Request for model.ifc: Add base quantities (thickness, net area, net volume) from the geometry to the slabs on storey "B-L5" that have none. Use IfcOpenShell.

First a look at what the model holds.

```python
import ifcopenshell
import ifcopenshell.util.element
import ifcopenshell.util.unit

model = ifcopenshell.open("model.ifc")
print(model.schema)
for unit_type in ("LENGTHUNIT", "AREAUNIT", "VOLUMEUNIT"):
    print(unit_type, ifcopenshell.util.unit.calculate_unit_scale(model, unit_type))
storey = next(s for s in model.by_type("IfcBuildingStorey") if s.Name == "B-L5")
slabs = [e for e in ifcopenshell.util.element.get_decomposition(storey) if e.is_a("IfcSlab")]
for e in sorted(slabs, key=lambda e: e.id()):
    print(e.id(), e.is_a(), e.Name, list(ifcopenshell.util.element.get_psets(e, qtos_only=True)), sep=" | ")
```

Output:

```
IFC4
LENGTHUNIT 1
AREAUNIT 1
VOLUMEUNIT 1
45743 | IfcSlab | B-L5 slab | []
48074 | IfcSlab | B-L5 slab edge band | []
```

```python
import ifcopenshell
import ifcopenshell.api.pset
import ifcopenshell.geom
import ifcopenshell.util.element
import ifcopenshell.util.shape
import ifcopenshell.util.unit

model = ifcopenshell.open("model.ifc")
unit_scale = ifcopenshell.util.unit.calculate_unit_scale(model)
area_scale = ifcopenshell.util.unit.calculate_unit_scale(model, "AREAUNIT")
volume_scale = ifcopenshell.util.unit.calculate_unit_scale(model, "VOLUMEUNIT")
settings = ifcopenshell.geom.settings()

storey = next(s for s in model.by_type("IfcBuildingStorey") if s.Name == "B-L5")
slabs = [e for e in ifcopenshell.util.element.get_decomposition(storey) if e.is_a("IfcSlab")]

for e in sorted(slabs, key=lambda e: e.id()):
    if ifcopenshell.util.element.get_psets(e, qtos_only=True, should_inherit=False):
        continue
    # Geometry comes back in metres, in the element's own axes.
    shape = ifcopenshell.geom.create_shape(settings, e)
    values = {
        "Width": ifcopenshell.util.shape.get_z(shape.geometry) / unit_scale,
        "NetArea": ifcopenshell.util.shape.get_footprint_area(shape.geometry) / area_scale,
        "NetVolume": ifcopenshell.util.shape.get_volume(shape.geometry) / volume_scale,
    }
    qto = ifcopenshell.api.pset.add_qto(model, product=e, name="Qto_SlabBaseQuantities")
    ifcopenshell.api.pset.edit_qto(model, qto=qto, properties=values)
    print(e.id(), {k: round(v, 3) for k, v in values.items()})

model.write("model_rev.ifc")
```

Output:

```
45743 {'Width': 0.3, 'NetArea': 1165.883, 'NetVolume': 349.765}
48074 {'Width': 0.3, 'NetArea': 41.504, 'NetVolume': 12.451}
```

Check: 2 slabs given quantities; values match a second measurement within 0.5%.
